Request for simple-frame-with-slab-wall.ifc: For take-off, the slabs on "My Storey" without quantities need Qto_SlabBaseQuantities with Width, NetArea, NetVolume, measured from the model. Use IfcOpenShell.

First a look at what the model holds.

```python
import ifcopenshell
import ifcopenshell.util.element
import ifcopenshell.util.unit

model = ifcopenshell.open("simple-frame-with-slab-wall.ifc")
print(model.schema)
for unit_type in ("LENGTHUNIT", "AREAUNIT", "VOLUMEUNIT"):
    print(unit_type, ifcopenshell.util.unit.calculate_unit_scale(model, unit_type))
storey = next(s for s in model.by_type("IfcBuildingStorey") if s.Name == "My Storey")
slabs = [e for e in ifcopenshell.util.element.get_decomposition(storey) if e.is_a("IfcSlab")]
for e in sorted(slabs, key=lambda e: e.id()):
    print(e.id(), e.is_a(), e.Name, list(ifcopenshell.util.element.get_psets(e, qtos_only=True)), sep=" | ")
```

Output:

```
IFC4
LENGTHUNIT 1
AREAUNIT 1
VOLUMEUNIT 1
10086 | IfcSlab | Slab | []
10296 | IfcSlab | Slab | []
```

```python
import ifcopenshell
import ifcopenshell.api.pset
import ifcopenshell.geom
import ifcopenshell.util.element
import ifcopenshell.util.shape
import ifcopenshell.util.unit

model = ifcopenshell.open("simple-frame-with-slab-wall.ifc")
unit_scale = ifcopenshell.util.unit.calculate_unit_scale(model)
area_scale = ifcopenshell.util.unit.calculate_unit_scale(model, "AREAUNIT")
volume_scale = ifcopenshell.util.unit.calculate_unit_scale(model, "VOLUMEUNIT")
settings = ifcopenshell.geom.settings()

storey = next(s for s in model.by_type("IfcBuildingStorey") if s.Name == "My Storey")
slabs = [e for e in ifcopenshell.util.element.get_decomposition(storey) if e.is_a("IfcSlab")]

for e in sorted(slabs, key=lambda e: e.id()):
    if ifcopenshell.util.element.get_psets(e, qtos_only=True, should_inherit=False):
        continue
    # Geometry comes back in metres, in the element's own axes.
    shape = ifcopenshell.geom.create_shape(settings, e)
    values = {
        "Width": ifcopenshell.util.shape.get_z(shape.geometry) / unit_scale,
        "NetArea": ifcopenshell.util.shape.get_footprint_area(shape.geometry) / area_scale,
        "NetVolume": ifcopenshell.util.shape.get_volume(shape.geometry) / volume_scale,
    }
    qto = ifcopenshell.api.pset.add_qto(model, product=e, name="Qto_SlabBaseQuantities")
    ifcopenshell.api.pset.edit_qto(model, qto=qto, properties=values)
    print(e.id(), {k: round(v, 3) for k, v in values.items()})

model.write("simple-frame-with-slab-wall_updated.ifc")
```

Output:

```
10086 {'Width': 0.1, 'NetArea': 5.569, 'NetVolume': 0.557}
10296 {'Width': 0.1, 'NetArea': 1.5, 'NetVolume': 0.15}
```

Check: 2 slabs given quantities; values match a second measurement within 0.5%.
